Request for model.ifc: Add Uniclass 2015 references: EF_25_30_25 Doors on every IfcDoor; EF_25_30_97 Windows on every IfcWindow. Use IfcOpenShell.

First a look at what the model holds.

```python
import ifcopenshell

model = ifcopenshell.open("model.ifc")
print(model.schema)
print("classifications:", [c.Name for c in model.by_type("IfcClassification")])
for ifc_class in ("IfcDoor", "IfcRoof", "IfcStair", "IfcWall", "IfcWindow"):
    print(ifc_class, len(model.by_type(ifc_class)))
```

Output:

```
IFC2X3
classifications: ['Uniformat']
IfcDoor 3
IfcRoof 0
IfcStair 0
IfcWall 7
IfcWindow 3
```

```python
import ifcopenshell
import ifcopenshell.api.classification

model = ifcopenshell.open("model.ifc")

# IFC2X3 requires Source and Edition and has no link from the project to the system.
system = model.create_entity("IfcClassification", Source="NBS", Edition="2015", Name="Uniclass 2015")

codes = {
    "IfcDoor": ("EF_25_30_25", "Doors"),
    "IfcWindow": ("EF_25_30_97", "Windows"),
}
for ifc_class, (code, name) in codes.items():
    products = model.by_type(ifc_class)
    ifcopenshell.api.classification.add_reference(
        model, products=products, classification=system, identification=code, name=name
    )
    print(code, len(products))

model.write("model_rev.ifc")
```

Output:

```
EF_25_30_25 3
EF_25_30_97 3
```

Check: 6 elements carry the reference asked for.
